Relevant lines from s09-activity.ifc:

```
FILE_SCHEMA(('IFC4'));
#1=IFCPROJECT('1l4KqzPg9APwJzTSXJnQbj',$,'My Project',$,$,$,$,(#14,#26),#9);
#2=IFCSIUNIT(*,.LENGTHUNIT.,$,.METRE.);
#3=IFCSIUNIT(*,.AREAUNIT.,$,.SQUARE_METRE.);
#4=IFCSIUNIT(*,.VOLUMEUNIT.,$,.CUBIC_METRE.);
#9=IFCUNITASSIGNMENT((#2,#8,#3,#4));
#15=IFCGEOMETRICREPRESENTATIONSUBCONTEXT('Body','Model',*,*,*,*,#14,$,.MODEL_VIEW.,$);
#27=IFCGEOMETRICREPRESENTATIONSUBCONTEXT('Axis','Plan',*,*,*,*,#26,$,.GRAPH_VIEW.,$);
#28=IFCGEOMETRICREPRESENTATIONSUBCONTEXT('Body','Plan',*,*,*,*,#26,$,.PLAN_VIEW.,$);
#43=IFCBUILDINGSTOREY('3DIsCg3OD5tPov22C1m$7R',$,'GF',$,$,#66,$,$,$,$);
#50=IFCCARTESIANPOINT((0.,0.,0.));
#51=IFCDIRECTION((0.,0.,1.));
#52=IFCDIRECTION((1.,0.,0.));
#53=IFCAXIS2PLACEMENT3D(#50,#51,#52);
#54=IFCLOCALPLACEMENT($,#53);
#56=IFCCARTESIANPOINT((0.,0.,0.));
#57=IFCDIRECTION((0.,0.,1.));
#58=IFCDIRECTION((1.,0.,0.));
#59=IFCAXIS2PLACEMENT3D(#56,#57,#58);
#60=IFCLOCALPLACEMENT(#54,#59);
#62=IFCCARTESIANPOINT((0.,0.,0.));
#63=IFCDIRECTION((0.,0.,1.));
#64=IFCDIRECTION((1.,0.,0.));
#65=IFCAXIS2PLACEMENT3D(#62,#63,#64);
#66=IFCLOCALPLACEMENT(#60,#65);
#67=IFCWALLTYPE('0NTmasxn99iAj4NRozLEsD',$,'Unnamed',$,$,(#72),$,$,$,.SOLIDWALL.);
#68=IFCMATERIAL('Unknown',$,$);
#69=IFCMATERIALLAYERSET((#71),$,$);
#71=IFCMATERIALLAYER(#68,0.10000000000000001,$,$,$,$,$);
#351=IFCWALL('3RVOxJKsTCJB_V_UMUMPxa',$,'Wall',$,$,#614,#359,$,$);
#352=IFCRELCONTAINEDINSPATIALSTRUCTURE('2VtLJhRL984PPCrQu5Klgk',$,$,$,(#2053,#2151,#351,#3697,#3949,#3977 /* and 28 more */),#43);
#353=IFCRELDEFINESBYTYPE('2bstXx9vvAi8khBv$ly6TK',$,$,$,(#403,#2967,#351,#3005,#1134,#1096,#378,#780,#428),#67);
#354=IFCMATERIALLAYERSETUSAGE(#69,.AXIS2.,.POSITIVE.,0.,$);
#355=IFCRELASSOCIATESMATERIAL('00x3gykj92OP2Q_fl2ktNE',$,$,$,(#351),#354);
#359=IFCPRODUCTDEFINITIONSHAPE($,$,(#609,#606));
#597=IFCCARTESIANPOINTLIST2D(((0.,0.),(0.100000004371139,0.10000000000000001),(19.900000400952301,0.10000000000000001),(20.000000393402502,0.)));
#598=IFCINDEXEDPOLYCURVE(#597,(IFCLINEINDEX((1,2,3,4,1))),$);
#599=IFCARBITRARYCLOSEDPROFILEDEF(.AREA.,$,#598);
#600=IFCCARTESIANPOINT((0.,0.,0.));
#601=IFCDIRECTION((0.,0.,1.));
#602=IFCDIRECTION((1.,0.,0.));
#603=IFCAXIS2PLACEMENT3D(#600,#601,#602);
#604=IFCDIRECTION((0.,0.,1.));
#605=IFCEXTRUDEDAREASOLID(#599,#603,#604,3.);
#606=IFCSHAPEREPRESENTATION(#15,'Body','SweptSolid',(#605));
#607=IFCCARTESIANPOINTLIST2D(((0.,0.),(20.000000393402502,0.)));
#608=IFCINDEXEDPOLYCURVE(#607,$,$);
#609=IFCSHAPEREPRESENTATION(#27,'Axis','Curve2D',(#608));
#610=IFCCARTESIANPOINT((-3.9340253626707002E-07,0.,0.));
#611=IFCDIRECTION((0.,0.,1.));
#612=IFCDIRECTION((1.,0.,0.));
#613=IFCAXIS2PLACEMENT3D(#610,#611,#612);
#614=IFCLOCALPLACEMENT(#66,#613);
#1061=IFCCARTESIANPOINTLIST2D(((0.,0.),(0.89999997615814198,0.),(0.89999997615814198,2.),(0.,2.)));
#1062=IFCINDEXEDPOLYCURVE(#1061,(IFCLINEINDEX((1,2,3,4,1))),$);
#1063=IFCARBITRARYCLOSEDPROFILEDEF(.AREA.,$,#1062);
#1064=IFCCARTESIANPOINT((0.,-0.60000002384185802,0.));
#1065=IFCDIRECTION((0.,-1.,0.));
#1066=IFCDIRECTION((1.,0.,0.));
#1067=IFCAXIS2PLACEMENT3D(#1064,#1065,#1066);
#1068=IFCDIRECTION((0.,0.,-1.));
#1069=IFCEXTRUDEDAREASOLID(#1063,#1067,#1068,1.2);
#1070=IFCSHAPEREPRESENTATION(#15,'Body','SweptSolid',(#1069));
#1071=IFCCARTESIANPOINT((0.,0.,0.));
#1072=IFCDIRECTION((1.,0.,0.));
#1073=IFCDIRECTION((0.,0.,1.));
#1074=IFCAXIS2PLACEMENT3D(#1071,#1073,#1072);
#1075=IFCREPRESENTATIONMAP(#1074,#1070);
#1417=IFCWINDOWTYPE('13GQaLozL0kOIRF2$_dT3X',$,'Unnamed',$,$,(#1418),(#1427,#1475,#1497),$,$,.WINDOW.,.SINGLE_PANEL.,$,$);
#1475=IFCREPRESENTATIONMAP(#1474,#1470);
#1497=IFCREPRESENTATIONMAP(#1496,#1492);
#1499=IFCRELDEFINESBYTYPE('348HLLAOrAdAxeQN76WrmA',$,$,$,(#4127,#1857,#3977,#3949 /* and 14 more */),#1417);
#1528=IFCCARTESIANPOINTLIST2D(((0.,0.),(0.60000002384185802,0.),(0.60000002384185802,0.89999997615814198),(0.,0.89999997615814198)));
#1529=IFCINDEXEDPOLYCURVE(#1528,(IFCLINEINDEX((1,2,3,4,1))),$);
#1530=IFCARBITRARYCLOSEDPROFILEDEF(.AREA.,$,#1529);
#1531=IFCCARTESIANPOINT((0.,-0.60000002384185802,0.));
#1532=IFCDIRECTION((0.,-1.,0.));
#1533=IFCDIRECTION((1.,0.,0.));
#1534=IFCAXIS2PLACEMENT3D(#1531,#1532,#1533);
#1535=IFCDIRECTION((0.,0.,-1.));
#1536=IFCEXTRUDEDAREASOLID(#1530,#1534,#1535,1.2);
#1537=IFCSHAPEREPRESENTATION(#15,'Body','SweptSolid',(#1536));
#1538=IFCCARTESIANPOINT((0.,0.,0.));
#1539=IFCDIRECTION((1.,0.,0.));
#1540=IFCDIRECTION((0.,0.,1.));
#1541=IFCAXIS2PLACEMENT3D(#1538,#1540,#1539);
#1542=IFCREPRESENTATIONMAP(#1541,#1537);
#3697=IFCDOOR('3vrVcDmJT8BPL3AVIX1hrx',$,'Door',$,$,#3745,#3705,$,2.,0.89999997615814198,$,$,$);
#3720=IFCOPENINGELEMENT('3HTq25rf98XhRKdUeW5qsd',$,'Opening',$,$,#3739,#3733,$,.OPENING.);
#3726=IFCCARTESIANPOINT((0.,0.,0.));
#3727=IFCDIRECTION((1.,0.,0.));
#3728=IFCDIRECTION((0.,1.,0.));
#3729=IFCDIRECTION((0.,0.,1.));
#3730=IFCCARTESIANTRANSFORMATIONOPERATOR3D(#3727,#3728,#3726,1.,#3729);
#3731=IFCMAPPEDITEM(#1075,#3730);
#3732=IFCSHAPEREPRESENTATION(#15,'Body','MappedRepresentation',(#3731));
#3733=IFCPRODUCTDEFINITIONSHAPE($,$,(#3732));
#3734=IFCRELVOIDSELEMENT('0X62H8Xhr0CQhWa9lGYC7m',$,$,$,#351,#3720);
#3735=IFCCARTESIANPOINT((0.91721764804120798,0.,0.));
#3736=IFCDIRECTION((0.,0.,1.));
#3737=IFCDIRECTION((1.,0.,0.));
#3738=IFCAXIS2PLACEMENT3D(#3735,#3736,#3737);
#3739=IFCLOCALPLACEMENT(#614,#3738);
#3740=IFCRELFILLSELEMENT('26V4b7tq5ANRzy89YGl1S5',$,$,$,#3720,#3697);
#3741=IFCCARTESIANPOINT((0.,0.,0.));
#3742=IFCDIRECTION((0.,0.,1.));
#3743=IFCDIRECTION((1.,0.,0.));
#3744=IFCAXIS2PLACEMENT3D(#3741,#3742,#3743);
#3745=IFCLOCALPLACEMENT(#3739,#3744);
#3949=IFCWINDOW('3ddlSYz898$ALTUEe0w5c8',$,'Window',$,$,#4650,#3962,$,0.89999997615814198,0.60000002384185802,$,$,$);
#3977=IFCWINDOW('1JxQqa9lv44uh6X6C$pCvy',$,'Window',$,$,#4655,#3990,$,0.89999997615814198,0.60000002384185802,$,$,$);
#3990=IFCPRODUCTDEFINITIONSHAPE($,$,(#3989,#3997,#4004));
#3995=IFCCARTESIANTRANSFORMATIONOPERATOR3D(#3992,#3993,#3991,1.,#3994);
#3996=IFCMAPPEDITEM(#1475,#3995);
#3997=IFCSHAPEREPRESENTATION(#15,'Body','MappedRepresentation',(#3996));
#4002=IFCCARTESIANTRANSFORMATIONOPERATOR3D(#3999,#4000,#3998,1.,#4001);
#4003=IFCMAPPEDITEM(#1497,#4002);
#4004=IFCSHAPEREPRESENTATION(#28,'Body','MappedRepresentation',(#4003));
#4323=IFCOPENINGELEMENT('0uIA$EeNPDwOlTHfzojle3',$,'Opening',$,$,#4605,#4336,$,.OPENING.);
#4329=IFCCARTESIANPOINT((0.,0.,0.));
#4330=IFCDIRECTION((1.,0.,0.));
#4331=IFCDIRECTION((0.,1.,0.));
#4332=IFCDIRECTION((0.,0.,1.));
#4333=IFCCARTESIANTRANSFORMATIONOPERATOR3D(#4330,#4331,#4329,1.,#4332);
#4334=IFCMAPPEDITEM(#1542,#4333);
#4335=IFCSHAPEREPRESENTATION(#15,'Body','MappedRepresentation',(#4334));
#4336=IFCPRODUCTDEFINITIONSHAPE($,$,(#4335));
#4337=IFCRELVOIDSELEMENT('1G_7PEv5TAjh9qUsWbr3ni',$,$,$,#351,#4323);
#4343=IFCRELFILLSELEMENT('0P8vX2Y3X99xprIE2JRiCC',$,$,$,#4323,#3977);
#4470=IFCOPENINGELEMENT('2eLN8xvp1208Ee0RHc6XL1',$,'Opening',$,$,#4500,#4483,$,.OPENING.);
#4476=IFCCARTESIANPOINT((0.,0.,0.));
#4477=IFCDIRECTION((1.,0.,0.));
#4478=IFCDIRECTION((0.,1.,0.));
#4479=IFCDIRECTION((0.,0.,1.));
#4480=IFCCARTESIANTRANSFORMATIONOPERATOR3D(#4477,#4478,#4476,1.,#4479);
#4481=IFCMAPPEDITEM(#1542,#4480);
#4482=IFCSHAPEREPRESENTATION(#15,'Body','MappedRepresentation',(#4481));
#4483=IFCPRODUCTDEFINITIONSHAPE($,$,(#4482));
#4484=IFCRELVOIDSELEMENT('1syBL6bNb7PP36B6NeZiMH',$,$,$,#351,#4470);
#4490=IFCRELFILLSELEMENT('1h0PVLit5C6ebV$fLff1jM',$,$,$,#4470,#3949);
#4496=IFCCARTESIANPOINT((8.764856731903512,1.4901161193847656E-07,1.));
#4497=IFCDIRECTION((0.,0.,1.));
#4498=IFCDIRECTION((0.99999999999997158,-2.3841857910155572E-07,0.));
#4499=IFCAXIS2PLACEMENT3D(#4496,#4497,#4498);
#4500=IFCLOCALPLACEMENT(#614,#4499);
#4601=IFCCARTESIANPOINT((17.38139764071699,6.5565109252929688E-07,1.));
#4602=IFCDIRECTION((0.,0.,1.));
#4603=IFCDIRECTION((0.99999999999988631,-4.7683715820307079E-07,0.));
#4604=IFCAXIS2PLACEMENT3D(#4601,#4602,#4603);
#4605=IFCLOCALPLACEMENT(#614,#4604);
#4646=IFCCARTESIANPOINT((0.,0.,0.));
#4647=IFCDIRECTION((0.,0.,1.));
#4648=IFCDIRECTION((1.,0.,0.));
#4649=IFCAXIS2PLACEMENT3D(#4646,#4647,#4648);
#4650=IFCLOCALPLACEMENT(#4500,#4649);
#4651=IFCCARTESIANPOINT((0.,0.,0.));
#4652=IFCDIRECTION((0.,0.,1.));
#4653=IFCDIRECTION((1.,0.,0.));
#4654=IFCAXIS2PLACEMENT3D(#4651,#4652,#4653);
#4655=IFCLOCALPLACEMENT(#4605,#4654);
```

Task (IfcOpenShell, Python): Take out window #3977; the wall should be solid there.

```python
import ifcopenshell
import ifcopenshell.api.feature
import ifcopenshell.api.root
import ifcopenshell.geom
import ifcopenshell.util.shape

model = ifcopenshell.open("s09-activity.ifc")
settings = ifcopenshell.geom.settings()


def volume(element):
    """Net volume in cubic metres, openings subtracted."""
    shape = ifcopenshell.geom.create_shape(settings, element)
    return ifcopenshell.util.shape.get_volume(shape.geometry)


window = model.by_id(3977)
opening = window.FillsVoids[0].RelatingOpeningElement
wall = opening.VoidsElements[0].RelatingBuildingElement
before = volume(wall)

ifcopenshell.api.root.remove_product(model, product=window)
ifcopenshell.api.feature.remove_feature(model, feature=opening)

after = volume(wall)

print(f"wall volume {before:.3f} -> {after:.3f} m3")

model.write("s09-activity_edited.ifc")
```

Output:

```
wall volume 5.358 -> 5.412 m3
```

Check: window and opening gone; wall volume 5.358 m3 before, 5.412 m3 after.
